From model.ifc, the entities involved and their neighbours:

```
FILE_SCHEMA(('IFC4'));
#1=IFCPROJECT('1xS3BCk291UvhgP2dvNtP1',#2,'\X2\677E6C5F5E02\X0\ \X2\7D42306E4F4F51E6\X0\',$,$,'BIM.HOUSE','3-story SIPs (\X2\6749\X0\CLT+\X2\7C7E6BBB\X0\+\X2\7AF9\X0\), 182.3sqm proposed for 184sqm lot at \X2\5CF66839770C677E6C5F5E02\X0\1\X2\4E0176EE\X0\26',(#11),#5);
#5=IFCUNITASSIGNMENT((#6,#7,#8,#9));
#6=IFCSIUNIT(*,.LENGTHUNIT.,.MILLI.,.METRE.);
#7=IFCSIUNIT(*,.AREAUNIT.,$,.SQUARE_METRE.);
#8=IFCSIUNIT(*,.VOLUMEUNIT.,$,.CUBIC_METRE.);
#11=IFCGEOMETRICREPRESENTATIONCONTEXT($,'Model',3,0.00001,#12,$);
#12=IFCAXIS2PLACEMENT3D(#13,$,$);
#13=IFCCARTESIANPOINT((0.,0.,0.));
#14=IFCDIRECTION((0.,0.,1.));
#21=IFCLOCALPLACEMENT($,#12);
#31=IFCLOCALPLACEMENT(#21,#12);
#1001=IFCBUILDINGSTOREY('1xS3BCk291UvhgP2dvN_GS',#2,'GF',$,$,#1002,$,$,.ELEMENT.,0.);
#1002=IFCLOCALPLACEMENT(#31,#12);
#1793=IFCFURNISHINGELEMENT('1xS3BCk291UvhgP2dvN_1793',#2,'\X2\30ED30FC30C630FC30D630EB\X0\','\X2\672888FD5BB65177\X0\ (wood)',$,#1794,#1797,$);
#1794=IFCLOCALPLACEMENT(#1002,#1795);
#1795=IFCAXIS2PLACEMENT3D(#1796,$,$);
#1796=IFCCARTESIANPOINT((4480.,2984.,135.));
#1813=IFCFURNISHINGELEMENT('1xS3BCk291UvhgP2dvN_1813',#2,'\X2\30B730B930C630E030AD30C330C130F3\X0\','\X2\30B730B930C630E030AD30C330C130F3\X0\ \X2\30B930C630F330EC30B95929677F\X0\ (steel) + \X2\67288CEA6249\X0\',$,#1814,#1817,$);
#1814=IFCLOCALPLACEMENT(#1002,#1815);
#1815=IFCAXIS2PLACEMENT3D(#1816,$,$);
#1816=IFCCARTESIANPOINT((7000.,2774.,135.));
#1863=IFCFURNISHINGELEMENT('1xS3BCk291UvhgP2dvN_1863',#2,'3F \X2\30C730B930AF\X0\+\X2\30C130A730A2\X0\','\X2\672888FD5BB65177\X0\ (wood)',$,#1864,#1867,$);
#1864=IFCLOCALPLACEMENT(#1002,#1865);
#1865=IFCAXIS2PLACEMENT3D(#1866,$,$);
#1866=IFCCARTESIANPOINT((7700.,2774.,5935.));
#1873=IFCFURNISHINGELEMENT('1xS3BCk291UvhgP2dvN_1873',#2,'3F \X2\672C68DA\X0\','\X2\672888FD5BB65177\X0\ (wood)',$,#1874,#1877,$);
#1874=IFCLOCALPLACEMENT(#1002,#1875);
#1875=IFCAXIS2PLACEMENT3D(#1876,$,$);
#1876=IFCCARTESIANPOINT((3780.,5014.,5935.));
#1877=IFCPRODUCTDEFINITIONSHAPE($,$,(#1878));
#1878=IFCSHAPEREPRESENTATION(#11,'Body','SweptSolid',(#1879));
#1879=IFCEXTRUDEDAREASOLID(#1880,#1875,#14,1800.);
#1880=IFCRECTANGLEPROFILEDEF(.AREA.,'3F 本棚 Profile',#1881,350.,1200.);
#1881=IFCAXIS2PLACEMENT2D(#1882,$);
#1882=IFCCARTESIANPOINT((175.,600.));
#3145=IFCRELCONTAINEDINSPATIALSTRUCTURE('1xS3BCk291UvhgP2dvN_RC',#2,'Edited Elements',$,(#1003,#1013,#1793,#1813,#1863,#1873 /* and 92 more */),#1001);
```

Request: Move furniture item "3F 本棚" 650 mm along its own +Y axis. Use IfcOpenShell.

```python
import ifcopenshell
import ifcopenshell.api.geometry
import ifcopenshell.util.placement

model = ifcopenshell.open("model.ifc")

item = model.by_id(1873)
matrix = ifcopenshell.util.placement.get_local_placement(item.ObjectPlacement)
matrix[:3, 3] += matrix[:3, 1] * 650.0
ifcopenshell.api.geometry.edit_object_placement(model, product=item, matrix=matrix, is_si=False)

print(ifcopenshell.util.placement.get_local_placement(item.ObjectPlacement).round(3) + 0.0)

model.write("model_edited.ifc")
```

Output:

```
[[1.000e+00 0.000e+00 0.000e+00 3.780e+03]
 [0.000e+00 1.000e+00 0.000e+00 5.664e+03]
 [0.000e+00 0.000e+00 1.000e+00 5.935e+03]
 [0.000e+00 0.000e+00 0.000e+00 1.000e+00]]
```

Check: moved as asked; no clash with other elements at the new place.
